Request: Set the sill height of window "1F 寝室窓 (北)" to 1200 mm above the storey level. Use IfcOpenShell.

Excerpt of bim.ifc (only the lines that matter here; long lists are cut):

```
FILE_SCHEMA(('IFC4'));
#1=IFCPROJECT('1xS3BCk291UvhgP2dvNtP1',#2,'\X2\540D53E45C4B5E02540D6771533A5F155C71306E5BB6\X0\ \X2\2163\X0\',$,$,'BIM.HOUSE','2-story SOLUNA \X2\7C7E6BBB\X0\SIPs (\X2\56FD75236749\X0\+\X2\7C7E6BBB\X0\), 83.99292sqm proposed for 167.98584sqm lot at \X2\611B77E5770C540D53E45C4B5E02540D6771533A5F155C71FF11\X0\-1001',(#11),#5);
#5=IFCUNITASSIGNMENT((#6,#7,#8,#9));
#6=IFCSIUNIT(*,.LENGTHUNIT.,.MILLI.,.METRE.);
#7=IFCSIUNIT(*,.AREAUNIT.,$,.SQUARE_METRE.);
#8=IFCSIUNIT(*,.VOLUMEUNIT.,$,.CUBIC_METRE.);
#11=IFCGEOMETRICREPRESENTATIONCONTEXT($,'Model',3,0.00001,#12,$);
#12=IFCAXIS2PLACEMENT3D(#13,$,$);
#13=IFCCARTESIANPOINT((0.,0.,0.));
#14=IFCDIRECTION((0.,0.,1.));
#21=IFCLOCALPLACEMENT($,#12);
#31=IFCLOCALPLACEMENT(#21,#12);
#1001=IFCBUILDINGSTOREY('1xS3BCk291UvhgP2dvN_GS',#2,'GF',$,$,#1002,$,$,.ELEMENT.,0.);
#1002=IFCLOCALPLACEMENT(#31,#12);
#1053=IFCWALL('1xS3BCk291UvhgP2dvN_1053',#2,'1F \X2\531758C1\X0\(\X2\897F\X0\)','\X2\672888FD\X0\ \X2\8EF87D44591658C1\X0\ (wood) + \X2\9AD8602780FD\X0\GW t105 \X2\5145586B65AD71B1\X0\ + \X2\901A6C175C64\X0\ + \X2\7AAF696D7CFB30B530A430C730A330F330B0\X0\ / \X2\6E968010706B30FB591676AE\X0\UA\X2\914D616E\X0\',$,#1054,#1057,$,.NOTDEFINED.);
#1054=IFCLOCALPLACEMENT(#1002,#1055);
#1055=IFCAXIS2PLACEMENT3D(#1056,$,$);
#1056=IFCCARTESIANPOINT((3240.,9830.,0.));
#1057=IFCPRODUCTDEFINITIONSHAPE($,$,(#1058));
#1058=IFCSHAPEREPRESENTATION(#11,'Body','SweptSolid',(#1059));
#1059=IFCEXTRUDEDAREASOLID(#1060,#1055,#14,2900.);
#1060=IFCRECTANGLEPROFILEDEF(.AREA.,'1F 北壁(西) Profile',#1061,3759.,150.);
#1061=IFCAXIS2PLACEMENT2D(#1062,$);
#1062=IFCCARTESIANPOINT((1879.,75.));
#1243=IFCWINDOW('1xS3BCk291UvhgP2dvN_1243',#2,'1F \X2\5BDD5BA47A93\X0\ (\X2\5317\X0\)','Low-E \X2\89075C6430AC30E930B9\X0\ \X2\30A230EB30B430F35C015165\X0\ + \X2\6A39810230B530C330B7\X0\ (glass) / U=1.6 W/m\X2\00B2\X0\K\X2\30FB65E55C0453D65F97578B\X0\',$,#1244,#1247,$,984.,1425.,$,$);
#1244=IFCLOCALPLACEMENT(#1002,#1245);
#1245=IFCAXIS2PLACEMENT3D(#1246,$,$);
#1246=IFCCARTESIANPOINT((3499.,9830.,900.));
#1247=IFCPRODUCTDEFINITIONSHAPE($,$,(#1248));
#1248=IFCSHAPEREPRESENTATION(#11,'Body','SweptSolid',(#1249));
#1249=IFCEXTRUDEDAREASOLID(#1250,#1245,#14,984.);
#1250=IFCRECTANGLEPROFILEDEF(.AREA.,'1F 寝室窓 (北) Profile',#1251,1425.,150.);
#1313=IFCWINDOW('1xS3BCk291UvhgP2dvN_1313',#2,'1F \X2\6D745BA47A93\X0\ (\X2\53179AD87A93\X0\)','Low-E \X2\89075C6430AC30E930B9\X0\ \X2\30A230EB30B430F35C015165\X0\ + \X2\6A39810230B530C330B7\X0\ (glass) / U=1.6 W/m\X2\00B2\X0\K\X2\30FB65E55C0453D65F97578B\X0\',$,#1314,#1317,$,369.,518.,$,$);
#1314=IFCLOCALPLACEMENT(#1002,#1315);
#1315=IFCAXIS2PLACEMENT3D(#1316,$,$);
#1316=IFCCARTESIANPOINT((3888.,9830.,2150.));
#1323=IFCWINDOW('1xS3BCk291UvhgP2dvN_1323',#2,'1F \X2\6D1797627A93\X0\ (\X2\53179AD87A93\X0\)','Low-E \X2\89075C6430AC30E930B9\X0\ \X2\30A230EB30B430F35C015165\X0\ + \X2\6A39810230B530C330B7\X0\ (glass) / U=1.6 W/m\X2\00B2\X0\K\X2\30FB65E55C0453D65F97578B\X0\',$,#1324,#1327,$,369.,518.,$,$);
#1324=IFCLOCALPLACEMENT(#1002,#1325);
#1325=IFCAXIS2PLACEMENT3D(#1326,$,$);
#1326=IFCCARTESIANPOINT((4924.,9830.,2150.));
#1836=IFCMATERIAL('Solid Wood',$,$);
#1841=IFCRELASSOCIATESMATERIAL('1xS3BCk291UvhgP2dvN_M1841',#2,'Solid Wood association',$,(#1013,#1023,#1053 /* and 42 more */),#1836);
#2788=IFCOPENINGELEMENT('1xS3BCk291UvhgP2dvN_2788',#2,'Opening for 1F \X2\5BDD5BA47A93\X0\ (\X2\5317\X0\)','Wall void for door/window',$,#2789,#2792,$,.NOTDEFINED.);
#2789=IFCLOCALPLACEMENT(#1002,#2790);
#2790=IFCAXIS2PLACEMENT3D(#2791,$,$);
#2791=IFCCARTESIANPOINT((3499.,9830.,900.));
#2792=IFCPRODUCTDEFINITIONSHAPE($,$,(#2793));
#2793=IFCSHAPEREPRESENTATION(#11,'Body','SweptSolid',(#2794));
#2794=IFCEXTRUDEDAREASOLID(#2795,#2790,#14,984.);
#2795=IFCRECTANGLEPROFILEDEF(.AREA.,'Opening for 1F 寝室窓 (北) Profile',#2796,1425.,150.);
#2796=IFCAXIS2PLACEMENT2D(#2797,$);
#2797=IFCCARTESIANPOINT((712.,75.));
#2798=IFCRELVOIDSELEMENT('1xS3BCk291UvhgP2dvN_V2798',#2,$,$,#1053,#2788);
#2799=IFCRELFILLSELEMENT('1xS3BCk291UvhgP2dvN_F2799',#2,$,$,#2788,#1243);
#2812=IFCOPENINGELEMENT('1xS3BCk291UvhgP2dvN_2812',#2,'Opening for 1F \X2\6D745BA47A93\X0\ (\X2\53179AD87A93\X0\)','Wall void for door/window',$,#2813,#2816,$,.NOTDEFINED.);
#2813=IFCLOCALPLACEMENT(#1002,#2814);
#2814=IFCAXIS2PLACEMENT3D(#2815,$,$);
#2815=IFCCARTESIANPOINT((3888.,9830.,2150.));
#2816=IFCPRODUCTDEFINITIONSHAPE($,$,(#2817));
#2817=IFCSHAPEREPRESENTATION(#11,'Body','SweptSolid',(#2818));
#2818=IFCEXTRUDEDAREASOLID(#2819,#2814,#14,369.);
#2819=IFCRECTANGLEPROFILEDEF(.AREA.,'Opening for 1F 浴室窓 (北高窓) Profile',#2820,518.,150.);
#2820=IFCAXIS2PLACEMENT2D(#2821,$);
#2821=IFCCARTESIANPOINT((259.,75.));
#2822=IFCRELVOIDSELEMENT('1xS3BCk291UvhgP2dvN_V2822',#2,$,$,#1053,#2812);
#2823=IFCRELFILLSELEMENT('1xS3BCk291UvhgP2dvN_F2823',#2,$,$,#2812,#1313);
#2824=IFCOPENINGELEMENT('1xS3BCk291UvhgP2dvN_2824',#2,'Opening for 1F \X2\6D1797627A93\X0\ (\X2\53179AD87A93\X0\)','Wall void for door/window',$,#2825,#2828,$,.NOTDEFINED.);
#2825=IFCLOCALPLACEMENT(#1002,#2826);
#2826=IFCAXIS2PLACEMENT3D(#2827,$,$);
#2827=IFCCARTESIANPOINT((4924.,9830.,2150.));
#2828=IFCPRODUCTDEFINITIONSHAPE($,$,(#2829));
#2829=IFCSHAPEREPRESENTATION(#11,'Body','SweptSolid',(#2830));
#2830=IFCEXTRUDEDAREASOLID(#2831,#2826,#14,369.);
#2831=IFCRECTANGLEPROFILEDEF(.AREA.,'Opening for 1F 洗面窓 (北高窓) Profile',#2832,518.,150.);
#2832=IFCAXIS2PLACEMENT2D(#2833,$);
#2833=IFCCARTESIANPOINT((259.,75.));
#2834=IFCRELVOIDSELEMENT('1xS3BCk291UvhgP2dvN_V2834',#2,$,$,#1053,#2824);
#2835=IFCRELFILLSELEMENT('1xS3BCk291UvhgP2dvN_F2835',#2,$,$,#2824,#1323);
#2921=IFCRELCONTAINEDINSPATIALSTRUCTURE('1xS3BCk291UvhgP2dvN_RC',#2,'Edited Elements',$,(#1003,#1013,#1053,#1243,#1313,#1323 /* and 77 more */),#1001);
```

```python
import numpy as np
import ifcopenshell
import ifcopenshell.api.geometry
import ifcopenshell.geom
import ifcopenshell.util.element
import ifcopenshell.util.placement
import ifcopenshell.util.shape
import ifcopenshell.util.unit

model = ifcopenshell.open("bim.ifc")
unit_scale = ifcopenshell.util.unit.calculate_unit_scale(model)

window = model.by_guid("1xS3BCk291UvhgP2dvN_1243")
opening = window.FillsVoids[0].RelatingOpeningElement
storey = ifcopenshell.util.element.get_container(window, ifc_class="IfcBuildingStorey")
level = ifcopenshell.util.placement.get_local_placement(storey.ObjectPlacement)[2, 3]

# The opening's origin need not be at the sill, so measure its lowest point.
shape = ifcopenshell.geom.create_shape(ifcopenshell.geom.settings(), opening)
bottom = ifcopenshell.util.shape.get_shape_bottom_elevation(shape, shape.geometry) / unit_scale
dz = level + 1200.0 - bottom

shift = np.array([0.0, 0.0, dz])
# The window is not placed relative to its opening, so move both.
for product in (opening, window):
    matrix = ifcopenshell.util.placement.get_local_placement(product.ObjectPlacement)
    matrix[:3, 3] += shift
    ifcopenshell.api.geometry.edit_object_placement(model, product=product, matrix=matrix, is_si=False)

print(f"moved by {dz * unit_scale:+.3f} m")

model.write("bim_v2.ifc")
```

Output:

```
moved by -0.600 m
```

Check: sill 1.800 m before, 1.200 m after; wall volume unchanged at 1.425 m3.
